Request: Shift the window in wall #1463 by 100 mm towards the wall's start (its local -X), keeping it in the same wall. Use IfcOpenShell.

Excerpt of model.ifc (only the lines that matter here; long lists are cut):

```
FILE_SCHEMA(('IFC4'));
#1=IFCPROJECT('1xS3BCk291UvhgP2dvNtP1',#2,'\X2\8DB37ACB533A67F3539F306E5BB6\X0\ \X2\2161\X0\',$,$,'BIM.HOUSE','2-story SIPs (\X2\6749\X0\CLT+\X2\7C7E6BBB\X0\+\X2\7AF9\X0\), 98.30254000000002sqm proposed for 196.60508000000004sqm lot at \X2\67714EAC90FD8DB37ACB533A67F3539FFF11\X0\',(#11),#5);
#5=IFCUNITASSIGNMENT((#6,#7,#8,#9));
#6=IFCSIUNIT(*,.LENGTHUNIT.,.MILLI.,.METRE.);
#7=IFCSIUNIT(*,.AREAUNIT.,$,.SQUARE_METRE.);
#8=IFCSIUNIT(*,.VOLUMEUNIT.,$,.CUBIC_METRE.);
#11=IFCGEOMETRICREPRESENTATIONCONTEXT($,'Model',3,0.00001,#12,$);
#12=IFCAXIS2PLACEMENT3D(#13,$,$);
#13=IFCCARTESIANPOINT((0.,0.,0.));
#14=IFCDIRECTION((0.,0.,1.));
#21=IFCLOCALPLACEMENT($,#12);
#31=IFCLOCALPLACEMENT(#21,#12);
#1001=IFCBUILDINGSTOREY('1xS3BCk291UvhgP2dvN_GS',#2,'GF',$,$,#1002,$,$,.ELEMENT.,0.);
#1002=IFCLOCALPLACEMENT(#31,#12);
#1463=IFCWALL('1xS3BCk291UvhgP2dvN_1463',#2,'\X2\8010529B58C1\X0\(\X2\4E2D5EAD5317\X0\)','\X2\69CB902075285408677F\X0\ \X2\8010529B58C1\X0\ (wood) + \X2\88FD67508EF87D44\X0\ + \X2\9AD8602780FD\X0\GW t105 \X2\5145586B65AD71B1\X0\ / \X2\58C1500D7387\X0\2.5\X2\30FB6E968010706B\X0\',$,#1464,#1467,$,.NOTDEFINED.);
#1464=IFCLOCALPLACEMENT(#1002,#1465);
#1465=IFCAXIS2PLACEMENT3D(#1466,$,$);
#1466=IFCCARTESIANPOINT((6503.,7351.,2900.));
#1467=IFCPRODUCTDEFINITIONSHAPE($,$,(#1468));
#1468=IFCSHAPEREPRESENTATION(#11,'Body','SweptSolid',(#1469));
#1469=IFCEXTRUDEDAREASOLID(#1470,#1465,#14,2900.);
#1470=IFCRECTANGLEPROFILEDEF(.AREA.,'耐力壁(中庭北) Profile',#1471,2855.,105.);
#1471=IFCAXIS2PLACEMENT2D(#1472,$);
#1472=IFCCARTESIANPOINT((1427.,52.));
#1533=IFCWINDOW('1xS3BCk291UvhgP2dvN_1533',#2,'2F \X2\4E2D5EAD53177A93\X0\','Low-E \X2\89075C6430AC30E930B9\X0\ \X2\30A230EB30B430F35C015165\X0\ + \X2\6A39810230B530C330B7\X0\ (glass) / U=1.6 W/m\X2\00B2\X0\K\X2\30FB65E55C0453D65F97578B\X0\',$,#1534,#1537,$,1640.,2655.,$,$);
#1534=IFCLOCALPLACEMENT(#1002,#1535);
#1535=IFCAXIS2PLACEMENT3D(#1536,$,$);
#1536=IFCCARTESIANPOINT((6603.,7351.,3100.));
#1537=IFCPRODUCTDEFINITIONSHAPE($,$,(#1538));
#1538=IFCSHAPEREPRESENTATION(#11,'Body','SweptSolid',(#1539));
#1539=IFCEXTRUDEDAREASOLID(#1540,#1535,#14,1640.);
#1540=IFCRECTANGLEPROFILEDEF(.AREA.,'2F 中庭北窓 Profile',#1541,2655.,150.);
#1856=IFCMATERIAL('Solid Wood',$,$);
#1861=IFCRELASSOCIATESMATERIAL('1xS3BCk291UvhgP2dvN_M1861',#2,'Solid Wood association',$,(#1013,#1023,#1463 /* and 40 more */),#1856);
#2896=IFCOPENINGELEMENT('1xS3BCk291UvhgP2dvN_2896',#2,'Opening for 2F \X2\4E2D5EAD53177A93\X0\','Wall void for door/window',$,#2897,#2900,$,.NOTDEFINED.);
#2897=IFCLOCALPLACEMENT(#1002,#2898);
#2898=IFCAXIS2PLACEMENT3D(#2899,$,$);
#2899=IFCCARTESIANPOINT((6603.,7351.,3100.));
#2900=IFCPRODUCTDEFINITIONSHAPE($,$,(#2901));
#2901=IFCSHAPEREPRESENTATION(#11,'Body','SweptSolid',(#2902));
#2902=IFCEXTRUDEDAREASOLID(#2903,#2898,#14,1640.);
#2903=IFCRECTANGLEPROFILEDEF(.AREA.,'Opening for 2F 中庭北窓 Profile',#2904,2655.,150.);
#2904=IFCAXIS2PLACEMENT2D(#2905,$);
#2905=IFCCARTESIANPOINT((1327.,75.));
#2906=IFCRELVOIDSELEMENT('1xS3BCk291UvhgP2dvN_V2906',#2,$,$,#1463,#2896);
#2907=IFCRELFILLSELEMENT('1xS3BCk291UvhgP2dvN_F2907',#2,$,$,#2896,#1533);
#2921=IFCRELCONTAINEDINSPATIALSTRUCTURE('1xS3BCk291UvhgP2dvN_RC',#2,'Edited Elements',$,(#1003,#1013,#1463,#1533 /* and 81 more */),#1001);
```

```python
import ifcopenshell
import ifcopenshell.api.geometry
import ifcopenshell.util.placement

model = ifcopenshell.open("model.ifc")

window = model.by_guid("1xS3BCk291UvhgP2dvN_1533")
opening = window.FillsVoids[0].RelatingOpeningElement
wall = opening.VoidsElements[0].RelatingBuildingElement

wall_matrix = ifcopenshell.util.placement.get_local_placement(wall.ObjectPlacement)
shift = wall_matrix[:3, 0] * -100.0
before = ifcopenshell.util.placement.get_local_placement(window.ObjectPlacement)[:3, 3].copy()

# The window is not placed relative to its opening, so move both.
for product in (opening, window):
    matrix = ifcopenshell.util.placement.get_local_placement(product.ObjectPlacement)
    matrix[:3, 3] += shift
    ifcopenshell.api.geometry.edit_object_placement(model, product=product, matrix=matrix, is_si=False)

after = ifcopenshell.util.placement.get_local_placement(window.ObjectPlacement)[:3, 3]
print("window moved by", (after - before).round(3) + 0.0)

model.write("model_rev.ifc")
```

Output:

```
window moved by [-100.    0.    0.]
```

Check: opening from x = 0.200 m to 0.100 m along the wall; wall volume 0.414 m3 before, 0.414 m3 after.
